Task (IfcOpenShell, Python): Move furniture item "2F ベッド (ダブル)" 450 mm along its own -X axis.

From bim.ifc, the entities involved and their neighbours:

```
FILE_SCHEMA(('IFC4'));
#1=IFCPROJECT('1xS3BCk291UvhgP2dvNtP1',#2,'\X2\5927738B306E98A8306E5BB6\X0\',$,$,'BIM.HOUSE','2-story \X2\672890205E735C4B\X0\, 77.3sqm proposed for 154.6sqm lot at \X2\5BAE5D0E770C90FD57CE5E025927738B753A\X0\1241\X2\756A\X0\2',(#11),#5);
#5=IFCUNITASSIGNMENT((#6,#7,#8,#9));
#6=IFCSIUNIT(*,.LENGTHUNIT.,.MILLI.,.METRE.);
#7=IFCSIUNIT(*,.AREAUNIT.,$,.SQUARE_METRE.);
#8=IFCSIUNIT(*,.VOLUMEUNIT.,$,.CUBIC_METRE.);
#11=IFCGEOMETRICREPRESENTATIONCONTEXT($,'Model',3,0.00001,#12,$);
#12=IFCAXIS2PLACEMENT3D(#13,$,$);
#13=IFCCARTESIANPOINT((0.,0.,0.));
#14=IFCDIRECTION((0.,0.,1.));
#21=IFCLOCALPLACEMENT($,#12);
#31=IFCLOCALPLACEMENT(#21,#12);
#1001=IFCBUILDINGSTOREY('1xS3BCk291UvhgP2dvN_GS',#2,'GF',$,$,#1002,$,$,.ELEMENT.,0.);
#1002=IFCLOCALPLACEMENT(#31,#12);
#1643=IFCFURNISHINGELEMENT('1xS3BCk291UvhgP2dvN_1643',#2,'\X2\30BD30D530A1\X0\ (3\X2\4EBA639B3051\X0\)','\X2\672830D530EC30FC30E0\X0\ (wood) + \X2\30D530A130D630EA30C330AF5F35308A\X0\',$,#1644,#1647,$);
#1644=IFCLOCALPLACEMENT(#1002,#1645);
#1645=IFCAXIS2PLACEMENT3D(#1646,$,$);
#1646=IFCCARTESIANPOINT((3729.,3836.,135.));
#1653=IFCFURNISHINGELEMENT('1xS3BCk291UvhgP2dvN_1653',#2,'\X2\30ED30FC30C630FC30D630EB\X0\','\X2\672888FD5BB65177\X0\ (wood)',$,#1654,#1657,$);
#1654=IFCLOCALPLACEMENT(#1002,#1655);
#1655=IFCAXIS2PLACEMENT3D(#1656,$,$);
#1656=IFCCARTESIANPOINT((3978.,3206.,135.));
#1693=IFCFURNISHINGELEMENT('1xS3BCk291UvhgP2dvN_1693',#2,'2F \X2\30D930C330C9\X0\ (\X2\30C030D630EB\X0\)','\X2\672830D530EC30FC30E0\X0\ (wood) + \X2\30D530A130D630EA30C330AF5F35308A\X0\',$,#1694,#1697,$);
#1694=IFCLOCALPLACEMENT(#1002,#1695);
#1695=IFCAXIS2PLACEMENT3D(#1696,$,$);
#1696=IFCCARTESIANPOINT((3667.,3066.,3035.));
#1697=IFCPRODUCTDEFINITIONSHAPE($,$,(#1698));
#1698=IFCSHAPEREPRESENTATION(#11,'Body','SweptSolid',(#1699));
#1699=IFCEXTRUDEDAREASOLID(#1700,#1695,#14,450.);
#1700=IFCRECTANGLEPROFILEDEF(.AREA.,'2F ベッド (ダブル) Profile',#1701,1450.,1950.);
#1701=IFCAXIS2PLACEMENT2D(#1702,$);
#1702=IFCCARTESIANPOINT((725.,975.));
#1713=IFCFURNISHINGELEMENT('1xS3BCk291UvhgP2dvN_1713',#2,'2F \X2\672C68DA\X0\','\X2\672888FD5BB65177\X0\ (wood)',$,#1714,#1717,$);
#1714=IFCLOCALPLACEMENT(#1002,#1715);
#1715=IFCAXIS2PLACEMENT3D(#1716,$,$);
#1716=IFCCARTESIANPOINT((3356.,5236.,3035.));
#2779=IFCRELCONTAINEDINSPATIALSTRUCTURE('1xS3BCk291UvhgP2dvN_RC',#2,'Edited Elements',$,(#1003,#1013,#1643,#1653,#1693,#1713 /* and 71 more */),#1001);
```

```python
import ifcopenshell
import ifcopenshell.api.geometry
import ifcopenshell.util.placement
import ifcopenshell.util.unit

model = ifcopenshell.open("bim.ifc")
unit_scale = ifcopenshell.util.unit.calculate_unit_scale(model)

item = model.by_guid("1xS3BCk291UvhgP2dvN_1693")
matrix = ifcopenshell.util.placement.get_local_placement(item.ObjectPlacement)
matrix[:3, 3] -= matrix[:3, 0] * 0.45 / unit_scale
ifcopenshell.api.geometry.edit_object_placement(model, product=item, matrix=matrix, is_si=False)

print(ifcopenshell.util.placement.get_local_placement(item.ObjectPlacement).round(3) + 0.0)

model.write("bim_edited.ifc")
```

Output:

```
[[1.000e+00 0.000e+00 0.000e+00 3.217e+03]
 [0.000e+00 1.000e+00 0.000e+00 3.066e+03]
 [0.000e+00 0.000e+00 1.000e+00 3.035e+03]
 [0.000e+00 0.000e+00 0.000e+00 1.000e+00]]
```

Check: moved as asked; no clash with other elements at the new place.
